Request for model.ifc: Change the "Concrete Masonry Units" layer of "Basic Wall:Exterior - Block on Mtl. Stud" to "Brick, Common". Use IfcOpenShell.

First a look at what the model holds.

```python
import ifcopenshell
import ifcopenshell.util.element

model = ifcopenshell.open("model.ifc")
print(model.schema)
for layer_set in model.by_type("IfcMaterialLayerSet"):
    if layer_set.LayerSetName == "Basic Wall:Exterior - Block on Mtl. Stud":
        for layer in layer_set.MaterialLayers:
            print(layer.id(), layer.Material and layer.Material.Name, layer.LayerThickness, sep=" | ")
        print(len(ifcopenshell.util.element.get_elements_by_material(model, layer_set)), "elements and types use it")
print(sorted(m.Name for m in model.by_type("IfcMaterial") if m.Name)[:60])
```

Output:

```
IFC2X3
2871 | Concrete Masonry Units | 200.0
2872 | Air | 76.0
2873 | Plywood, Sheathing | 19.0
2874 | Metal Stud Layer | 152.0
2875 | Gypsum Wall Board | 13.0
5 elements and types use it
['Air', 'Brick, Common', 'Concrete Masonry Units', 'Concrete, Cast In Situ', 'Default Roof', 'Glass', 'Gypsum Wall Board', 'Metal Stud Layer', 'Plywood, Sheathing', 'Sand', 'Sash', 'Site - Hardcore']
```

```python
import ifcopenshell
import ifcopenshell.api.material

model = ifcopenshell.open("model.ifc")

layer_set = next(s for s in model.by_type("IfcMaterialLayerSet") if s.LayerSetName == "Basic Wall:Exterior - Block on Mtl. Stud")
layer = next(l for l in layer_set.MaterialLayers if l.Material and l.Material.Name == "Concrete Masonry Units")
material = next(m for m in model.by_type("IfcMaterial") if m.Name == "Brick, Common")

# Point this one layer at the other material; renaming the old one would change it everywhere.
ifcopenshell.api.material.edit_layer(model, layer=layer, attributes={}, material=material)

print([l.Material.Name if l.Material else None for l in layer_set.MaterialLayers])

model.write("model_edited.ifc")
```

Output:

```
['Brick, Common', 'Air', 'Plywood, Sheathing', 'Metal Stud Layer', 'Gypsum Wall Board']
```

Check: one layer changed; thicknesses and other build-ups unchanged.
